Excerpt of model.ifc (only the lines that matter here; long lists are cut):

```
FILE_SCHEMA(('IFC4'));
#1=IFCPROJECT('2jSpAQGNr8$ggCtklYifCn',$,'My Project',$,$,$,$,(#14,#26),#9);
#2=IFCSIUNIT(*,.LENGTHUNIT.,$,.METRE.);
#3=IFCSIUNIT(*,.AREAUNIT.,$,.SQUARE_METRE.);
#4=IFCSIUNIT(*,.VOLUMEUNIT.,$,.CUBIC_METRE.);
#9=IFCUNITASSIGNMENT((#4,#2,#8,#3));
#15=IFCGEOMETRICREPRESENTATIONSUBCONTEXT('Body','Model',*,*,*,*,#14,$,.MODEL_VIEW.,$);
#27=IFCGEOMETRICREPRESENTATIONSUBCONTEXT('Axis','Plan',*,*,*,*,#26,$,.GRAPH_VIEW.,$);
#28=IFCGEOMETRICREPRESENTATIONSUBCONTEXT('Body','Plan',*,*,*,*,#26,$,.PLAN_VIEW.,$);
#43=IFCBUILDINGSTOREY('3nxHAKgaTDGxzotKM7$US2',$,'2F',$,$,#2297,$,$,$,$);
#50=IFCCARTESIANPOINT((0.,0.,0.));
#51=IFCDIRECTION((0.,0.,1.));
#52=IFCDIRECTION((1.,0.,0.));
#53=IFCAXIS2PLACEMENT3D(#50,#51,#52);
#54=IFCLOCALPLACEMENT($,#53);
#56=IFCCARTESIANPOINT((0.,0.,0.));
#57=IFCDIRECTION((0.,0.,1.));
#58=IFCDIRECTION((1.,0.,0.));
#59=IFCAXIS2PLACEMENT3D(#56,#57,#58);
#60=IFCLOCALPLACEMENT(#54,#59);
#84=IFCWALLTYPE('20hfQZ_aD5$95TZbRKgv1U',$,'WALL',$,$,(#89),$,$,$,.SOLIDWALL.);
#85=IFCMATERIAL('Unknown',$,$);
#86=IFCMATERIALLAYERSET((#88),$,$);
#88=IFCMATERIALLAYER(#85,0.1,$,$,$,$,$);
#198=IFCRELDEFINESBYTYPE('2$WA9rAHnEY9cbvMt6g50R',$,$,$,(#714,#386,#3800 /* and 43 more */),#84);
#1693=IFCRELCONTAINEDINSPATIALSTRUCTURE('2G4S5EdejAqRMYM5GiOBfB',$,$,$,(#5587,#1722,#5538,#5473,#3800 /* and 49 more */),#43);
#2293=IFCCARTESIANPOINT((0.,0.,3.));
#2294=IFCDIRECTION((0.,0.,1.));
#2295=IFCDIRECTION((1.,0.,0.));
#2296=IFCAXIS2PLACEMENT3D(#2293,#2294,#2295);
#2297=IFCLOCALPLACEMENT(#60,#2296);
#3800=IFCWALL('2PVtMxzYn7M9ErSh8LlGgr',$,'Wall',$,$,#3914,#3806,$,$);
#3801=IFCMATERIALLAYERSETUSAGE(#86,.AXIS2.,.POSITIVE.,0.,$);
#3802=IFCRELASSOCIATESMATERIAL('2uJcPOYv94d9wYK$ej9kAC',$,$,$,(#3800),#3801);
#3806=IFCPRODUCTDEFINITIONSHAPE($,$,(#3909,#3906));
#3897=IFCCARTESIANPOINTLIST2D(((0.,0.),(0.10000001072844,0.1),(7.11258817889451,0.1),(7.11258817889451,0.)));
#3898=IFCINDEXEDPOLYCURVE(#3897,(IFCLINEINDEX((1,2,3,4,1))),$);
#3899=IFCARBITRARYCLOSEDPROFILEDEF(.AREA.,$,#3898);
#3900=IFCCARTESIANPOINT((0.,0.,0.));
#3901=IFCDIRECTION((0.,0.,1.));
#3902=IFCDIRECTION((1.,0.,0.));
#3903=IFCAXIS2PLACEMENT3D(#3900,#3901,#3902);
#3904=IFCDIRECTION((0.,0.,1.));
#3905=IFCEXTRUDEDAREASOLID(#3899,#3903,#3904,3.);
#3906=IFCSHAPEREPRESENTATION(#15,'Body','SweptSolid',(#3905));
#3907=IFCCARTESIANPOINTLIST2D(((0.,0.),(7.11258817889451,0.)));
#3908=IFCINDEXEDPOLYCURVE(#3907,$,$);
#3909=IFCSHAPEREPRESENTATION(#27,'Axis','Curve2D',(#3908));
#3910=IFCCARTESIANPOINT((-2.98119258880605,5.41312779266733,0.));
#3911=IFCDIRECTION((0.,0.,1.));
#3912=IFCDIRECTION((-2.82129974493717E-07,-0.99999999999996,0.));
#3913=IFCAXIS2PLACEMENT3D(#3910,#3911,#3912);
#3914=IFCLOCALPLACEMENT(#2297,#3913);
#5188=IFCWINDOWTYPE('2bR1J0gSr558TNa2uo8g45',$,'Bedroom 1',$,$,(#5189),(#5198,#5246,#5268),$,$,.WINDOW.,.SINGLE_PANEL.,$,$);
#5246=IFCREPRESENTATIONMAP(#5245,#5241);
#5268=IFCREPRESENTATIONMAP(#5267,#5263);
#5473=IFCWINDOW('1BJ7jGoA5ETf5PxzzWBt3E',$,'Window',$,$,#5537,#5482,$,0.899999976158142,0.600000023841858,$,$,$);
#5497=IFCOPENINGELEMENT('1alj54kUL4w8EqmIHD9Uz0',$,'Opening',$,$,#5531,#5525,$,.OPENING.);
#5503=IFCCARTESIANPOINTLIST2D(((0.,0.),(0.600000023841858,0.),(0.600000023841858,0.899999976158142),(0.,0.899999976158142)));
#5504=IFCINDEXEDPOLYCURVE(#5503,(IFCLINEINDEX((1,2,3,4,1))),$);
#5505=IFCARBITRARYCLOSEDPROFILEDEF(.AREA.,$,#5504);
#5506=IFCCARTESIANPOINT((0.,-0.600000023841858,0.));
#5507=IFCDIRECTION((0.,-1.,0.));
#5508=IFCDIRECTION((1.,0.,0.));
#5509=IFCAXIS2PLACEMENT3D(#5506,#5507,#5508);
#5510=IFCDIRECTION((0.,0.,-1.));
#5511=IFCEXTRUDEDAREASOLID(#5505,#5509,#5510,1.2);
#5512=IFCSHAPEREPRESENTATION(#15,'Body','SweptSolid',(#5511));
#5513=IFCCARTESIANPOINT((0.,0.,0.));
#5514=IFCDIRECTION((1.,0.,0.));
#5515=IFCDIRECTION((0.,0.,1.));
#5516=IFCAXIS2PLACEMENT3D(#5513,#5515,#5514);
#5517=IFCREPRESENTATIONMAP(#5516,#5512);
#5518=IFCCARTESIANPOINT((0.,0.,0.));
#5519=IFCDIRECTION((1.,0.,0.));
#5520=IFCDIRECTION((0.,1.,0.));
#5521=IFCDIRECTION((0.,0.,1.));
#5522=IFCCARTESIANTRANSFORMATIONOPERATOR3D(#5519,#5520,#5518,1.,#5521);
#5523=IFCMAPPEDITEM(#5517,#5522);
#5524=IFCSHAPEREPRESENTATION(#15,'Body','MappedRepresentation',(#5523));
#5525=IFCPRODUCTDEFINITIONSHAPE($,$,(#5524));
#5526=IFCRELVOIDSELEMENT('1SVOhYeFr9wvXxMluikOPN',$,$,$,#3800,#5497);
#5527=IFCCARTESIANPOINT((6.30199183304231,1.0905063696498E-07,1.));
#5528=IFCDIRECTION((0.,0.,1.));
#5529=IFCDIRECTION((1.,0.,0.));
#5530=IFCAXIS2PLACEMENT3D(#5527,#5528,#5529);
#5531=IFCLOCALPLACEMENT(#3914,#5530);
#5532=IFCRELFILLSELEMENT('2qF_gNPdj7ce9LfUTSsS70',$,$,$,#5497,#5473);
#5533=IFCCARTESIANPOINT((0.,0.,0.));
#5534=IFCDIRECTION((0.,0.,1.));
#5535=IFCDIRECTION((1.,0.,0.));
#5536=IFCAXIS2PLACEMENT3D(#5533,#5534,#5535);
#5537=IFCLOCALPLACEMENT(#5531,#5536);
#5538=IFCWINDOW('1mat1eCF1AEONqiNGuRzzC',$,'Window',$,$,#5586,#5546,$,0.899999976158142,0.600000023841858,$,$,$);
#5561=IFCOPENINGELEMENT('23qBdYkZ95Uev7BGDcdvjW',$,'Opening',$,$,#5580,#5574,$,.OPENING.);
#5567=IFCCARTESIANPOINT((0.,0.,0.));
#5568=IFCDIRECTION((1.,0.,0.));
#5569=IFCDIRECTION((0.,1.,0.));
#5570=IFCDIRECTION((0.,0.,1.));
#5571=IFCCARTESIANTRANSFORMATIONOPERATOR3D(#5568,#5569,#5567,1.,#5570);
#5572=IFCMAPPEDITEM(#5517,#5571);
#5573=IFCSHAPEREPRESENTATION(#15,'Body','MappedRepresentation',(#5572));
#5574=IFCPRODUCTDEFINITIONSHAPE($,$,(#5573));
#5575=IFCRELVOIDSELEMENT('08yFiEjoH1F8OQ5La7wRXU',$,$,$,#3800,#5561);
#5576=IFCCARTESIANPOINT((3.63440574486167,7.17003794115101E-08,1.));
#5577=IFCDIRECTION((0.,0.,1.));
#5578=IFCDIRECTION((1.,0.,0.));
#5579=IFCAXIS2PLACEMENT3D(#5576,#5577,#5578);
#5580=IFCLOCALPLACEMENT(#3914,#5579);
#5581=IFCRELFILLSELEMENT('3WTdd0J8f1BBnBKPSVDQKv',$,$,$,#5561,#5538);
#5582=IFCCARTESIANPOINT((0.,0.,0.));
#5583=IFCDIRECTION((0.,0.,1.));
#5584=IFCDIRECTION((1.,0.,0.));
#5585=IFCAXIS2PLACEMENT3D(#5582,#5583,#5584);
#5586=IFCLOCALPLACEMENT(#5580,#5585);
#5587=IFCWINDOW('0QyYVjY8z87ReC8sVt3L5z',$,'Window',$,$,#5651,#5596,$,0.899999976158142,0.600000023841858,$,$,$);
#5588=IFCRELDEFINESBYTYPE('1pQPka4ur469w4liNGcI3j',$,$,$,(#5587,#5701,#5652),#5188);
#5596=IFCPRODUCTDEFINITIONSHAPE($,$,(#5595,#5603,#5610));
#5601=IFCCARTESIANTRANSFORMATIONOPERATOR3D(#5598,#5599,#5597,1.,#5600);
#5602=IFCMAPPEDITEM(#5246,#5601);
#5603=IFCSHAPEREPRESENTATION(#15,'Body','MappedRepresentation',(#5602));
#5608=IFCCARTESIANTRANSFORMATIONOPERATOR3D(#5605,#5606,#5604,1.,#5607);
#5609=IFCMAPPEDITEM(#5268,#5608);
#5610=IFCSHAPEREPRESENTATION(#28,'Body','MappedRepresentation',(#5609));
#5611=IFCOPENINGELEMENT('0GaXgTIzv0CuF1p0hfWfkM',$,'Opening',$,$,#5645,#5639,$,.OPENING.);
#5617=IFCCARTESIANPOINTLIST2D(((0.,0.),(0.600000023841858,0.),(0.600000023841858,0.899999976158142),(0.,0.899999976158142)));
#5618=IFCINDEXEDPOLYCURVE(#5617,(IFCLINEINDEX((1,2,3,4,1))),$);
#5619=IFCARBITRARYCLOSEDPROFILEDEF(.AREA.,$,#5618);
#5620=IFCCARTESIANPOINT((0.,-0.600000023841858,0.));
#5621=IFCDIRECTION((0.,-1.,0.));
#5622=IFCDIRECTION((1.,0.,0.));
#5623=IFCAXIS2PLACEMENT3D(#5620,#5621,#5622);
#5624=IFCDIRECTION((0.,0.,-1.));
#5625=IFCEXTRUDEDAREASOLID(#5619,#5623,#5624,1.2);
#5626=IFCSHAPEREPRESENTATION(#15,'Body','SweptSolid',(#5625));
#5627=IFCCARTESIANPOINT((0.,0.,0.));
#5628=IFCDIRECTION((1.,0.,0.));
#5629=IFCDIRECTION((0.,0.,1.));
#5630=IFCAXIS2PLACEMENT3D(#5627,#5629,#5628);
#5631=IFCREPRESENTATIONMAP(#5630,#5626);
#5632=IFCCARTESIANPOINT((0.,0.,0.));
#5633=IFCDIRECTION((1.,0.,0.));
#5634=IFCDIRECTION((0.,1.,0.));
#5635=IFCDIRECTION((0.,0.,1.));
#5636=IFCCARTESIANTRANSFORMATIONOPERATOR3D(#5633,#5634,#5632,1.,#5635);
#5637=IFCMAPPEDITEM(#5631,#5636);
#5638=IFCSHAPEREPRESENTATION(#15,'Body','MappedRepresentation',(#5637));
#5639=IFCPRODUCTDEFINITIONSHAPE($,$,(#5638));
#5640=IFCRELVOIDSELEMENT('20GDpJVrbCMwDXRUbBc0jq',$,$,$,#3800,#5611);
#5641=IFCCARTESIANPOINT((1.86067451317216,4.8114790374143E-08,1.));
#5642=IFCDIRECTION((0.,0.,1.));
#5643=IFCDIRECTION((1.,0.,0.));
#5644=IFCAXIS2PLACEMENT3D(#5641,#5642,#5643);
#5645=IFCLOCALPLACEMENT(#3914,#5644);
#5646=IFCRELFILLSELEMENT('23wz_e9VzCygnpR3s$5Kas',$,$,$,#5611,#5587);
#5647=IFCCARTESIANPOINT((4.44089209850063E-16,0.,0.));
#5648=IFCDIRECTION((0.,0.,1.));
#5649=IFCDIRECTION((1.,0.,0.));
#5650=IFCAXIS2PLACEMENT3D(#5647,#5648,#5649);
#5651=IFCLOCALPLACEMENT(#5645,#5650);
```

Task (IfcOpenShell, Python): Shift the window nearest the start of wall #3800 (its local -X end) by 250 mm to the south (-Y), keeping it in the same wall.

```python
import ifcopenshell
import ifcopenshell.api.geometry
import ifcopenshell.util.placement

model = ifcopenshell.open("model.ifc")

window = model.by_id(5587)
opening = window.FillsVoids[0].RelatingOpeningElement
wall = opening.VoidsElements[0].RelatingBuildingElement

wall_matrix = ifcopenshell.util.placement.get_local_placement(wall.ObjectPlacement)
shift = wall_matrix[:3, 0] * 0.25
before = ifcopenshell.util.placement.get_local_placement(window.ObjectPlacement)[:3, 3].copy()

# The window is placed relative to its opening, so it follows when the opening moves.
matrix = ifcopenshell.util.placement.get_local_placement(opening.ObjectPlacement)
matrix[:3, 3] += shift
ifcopenshell.api.geometry.edit_object_placement(
    model, product=opening, matrix=matrix, is_si=False, should_transform_children=True
)

after = ifcopenshell.util.placement.get_local_placement(window.ObjectPlacement)[:3, 3]
print("window moved by", (after - before).round(3) + 0.0)

model.write("model-out.ifc")
```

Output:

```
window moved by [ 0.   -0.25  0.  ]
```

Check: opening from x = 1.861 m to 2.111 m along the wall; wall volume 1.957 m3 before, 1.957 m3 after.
